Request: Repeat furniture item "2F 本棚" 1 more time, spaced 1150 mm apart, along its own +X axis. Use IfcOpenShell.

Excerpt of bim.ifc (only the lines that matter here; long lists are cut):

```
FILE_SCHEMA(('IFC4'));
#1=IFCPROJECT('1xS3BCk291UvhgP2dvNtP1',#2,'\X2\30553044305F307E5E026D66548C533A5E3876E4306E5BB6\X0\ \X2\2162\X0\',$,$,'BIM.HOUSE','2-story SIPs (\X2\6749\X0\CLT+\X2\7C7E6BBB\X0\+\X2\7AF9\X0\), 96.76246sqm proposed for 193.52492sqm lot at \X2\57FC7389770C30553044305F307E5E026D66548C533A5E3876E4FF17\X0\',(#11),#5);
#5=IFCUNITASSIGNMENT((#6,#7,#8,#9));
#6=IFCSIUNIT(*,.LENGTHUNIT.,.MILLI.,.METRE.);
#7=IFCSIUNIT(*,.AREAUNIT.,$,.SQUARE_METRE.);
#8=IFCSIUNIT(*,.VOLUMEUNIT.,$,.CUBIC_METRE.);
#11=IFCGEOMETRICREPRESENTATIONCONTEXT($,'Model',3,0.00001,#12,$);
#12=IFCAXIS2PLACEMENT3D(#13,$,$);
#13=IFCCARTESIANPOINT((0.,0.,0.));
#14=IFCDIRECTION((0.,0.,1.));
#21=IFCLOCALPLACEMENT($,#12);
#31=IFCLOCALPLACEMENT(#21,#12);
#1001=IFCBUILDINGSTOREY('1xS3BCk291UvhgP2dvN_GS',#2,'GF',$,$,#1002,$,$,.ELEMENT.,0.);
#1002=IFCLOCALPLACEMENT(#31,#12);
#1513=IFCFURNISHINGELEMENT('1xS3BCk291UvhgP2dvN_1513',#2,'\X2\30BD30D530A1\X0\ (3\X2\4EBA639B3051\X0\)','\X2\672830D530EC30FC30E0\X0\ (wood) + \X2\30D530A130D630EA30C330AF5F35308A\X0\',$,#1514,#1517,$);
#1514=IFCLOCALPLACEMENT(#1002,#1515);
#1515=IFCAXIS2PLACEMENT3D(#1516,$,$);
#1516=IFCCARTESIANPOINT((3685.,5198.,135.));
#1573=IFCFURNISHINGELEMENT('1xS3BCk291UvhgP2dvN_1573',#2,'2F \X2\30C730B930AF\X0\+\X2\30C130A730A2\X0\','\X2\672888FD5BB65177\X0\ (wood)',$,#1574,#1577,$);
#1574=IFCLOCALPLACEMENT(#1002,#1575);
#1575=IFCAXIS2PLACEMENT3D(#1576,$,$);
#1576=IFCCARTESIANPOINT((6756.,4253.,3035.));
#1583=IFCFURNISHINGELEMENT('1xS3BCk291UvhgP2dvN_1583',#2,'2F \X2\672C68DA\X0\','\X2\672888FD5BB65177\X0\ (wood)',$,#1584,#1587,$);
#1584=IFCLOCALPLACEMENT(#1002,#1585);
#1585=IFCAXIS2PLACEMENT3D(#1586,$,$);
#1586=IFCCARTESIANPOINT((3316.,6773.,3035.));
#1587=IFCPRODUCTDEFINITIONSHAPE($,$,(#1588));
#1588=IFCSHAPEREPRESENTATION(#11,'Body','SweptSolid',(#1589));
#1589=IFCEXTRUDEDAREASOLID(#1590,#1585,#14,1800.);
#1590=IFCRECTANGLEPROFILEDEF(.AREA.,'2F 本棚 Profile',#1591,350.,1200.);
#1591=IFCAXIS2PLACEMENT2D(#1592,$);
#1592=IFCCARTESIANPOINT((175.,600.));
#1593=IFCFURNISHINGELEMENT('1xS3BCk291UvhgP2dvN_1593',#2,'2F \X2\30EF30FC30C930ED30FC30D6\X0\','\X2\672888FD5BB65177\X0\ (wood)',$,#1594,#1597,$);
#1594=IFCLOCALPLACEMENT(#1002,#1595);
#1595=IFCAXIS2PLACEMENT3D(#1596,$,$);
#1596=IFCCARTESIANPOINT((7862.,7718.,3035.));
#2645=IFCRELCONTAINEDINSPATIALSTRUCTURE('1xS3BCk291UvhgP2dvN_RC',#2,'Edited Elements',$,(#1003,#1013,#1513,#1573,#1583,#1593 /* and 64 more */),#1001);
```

```python
import ifcopenshell
import ifcopenshell.api.geometry
import ifcopenshell.api.root
import ifcopenshell.util.element
import ifcopenshell.util.placement

model = ifcopenshell.open("bim.ifc")


def reuse_history(source, copy):
    """copy_class also copies each property set's owner history, people and application; keep the originals."""
    for rel in copy.IsDefinedBy:
        if rel.is_a("IfcRelDefinesByProperties") and (history := rel.RelatingPropertyDefinition.OwnerHistory):
            rel.RelatingPropertyDefinition.OwnerHistory = source.OwnerHistory
            ifcopenshell.util.element.remove_deep2(model, history)


source = model.by_guid("1xS3BCk291UvhgP2dvN_1583")
base = ifcopenshell.util.placement.get_local_placement(source.ObjectPlacement)
step = base[:3, 0] * 1150.0

for i in range(1, 2):
    copy = ifcopenshell.api.root.copy_class(model, product=source)
    copy.Representation = ifcopenshell.util.element.copy_deep(
        model, source.Representation, exclude=["IfcGeometricRepresentationContext", "IfcRepresentationMap"]
    )
    reuse_history(source, copy)
    matrix = base.copy()
    matrix[:3, 3] += i * step
    print("added at", matrix[:3, 3].round(3) + 0.0)
    ifcopenshell.api.geometry.edit_object_placement(model, product=copy, matrix=matrix, is_si=False)

model.write("bim-out.ifc")
```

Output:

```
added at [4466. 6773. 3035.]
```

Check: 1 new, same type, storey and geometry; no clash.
